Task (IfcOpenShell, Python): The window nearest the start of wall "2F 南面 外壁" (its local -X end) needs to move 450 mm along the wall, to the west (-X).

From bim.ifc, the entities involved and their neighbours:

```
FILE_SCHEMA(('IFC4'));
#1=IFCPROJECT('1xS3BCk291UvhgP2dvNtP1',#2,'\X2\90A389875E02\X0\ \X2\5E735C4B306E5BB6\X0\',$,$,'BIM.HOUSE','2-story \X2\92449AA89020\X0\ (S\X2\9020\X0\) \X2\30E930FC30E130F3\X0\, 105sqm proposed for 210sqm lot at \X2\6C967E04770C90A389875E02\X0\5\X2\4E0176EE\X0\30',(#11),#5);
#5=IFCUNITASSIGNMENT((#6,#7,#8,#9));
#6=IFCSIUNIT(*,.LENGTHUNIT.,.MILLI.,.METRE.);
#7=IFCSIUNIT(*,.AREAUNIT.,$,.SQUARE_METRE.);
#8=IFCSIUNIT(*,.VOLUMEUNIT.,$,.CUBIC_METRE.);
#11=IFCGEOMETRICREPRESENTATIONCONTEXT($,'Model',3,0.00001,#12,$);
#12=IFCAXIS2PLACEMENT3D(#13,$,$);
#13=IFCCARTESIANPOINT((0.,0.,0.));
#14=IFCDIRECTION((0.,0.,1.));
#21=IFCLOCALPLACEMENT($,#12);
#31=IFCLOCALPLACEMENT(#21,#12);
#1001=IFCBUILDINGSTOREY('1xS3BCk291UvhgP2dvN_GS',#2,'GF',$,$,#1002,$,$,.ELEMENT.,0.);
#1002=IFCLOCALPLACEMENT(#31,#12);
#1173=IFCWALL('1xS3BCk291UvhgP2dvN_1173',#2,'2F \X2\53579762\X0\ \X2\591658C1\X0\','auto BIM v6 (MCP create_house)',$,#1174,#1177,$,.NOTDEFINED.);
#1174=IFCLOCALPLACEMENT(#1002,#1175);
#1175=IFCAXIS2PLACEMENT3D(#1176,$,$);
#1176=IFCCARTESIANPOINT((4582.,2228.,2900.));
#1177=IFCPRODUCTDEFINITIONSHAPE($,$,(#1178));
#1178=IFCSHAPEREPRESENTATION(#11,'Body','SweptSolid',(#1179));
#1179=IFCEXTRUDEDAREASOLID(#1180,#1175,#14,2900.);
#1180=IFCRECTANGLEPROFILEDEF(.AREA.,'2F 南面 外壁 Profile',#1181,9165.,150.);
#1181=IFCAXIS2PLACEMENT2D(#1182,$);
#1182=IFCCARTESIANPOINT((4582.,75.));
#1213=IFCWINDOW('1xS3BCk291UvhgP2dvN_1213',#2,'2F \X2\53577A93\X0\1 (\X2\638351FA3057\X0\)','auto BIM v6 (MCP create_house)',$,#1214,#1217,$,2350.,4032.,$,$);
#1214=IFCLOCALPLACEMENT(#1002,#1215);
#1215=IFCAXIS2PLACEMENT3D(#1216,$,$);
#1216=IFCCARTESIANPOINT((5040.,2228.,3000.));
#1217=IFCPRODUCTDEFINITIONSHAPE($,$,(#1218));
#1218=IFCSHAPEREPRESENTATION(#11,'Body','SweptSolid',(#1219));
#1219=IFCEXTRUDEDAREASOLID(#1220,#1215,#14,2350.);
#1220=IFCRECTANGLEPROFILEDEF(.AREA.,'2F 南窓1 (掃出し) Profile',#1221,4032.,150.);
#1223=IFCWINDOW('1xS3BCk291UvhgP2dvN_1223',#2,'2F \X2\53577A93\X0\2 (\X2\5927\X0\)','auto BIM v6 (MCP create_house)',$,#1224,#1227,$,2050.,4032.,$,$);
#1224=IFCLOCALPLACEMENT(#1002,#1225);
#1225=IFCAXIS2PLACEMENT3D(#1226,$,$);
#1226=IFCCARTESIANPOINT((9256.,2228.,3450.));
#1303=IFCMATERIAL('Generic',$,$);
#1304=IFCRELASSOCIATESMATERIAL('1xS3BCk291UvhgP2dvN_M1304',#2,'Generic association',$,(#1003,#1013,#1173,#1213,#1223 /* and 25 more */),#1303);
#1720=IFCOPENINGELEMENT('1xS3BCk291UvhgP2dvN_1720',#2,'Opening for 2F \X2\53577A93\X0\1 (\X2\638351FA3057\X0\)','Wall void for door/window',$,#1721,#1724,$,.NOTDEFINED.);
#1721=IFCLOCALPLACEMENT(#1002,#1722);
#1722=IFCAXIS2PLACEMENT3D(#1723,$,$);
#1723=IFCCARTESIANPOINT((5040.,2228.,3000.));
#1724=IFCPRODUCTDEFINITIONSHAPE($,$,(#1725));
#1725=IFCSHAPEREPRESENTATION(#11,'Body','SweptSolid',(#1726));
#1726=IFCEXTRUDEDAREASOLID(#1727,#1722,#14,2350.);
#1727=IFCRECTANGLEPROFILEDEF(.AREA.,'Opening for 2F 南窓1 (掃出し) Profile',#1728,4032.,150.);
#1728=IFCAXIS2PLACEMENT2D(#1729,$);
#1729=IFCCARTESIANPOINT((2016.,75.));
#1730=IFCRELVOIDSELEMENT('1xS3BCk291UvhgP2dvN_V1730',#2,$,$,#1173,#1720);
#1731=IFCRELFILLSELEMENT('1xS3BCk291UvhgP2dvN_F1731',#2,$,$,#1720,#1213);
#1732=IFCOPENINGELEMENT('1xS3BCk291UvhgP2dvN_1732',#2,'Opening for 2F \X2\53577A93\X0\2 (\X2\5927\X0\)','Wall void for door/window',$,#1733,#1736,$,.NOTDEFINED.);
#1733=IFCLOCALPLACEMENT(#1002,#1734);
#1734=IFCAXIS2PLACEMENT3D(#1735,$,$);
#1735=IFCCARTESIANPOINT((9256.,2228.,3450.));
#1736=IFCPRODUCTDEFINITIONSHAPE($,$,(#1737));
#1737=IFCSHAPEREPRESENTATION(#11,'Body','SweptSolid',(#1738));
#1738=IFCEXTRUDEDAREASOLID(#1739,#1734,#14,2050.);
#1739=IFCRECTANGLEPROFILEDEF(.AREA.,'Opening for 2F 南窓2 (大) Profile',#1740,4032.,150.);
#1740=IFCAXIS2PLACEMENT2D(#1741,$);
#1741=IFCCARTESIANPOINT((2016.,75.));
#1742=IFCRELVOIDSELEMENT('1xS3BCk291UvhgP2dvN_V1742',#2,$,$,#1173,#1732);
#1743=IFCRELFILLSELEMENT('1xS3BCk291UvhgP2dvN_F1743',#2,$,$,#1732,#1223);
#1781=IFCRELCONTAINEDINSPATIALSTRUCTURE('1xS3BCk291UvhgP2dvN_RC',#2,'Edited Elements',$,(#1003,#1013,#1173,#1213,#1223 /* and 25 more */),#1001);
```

```python
import ifcopenshell
import ifcopenshell.api.geometry
import ifcopenshell.util.placement
import ifcopenshell.util.unit

model = ifcopenshell.open("bim.ifc")
unit_scale = ifcopenshell.util.unit.calculate_unit_scale(model)

window = model.by_guid("1xS3BCk291UvhgP2dvN_1213")
opening = window.FillsVoids[0].RelatingOpeningElement
wall = opening.VoidsElements[0].RelatingBuildingElement

wall_matrix = ifcopenshell.util.placement.get_local_placement(wall.ObjectPlacement)
shift = wall_matrix[:3, 0] * -0.45 / unit_scale
before = ifcopenshell.util.placement.get_local_placement(window.ObjectPlacement)[:3, 3].copy()

# The window is not placed relative to its opening, so move both.
for product in (opening, window):
    matrix = ifcopenshell.util.placement.get_local_placement(product.ObjectPlacement)
    matrix[:3, 3] += shift
    ifcopenshell.api.geometry.edit_object_placement(model, product=product, matrix=matrix, is_si=False)

after = ifcopenshell.util.placement.get_local_placement(window.ObjectPlacement)[:3, 3]
print("window moved by", (after - before).round(3) + 0.0)

model.write("bim_rev.ifc")
```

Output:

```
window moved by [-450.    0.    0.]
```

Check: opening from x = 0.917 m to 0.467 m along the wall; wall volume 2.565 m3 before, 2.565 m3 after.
